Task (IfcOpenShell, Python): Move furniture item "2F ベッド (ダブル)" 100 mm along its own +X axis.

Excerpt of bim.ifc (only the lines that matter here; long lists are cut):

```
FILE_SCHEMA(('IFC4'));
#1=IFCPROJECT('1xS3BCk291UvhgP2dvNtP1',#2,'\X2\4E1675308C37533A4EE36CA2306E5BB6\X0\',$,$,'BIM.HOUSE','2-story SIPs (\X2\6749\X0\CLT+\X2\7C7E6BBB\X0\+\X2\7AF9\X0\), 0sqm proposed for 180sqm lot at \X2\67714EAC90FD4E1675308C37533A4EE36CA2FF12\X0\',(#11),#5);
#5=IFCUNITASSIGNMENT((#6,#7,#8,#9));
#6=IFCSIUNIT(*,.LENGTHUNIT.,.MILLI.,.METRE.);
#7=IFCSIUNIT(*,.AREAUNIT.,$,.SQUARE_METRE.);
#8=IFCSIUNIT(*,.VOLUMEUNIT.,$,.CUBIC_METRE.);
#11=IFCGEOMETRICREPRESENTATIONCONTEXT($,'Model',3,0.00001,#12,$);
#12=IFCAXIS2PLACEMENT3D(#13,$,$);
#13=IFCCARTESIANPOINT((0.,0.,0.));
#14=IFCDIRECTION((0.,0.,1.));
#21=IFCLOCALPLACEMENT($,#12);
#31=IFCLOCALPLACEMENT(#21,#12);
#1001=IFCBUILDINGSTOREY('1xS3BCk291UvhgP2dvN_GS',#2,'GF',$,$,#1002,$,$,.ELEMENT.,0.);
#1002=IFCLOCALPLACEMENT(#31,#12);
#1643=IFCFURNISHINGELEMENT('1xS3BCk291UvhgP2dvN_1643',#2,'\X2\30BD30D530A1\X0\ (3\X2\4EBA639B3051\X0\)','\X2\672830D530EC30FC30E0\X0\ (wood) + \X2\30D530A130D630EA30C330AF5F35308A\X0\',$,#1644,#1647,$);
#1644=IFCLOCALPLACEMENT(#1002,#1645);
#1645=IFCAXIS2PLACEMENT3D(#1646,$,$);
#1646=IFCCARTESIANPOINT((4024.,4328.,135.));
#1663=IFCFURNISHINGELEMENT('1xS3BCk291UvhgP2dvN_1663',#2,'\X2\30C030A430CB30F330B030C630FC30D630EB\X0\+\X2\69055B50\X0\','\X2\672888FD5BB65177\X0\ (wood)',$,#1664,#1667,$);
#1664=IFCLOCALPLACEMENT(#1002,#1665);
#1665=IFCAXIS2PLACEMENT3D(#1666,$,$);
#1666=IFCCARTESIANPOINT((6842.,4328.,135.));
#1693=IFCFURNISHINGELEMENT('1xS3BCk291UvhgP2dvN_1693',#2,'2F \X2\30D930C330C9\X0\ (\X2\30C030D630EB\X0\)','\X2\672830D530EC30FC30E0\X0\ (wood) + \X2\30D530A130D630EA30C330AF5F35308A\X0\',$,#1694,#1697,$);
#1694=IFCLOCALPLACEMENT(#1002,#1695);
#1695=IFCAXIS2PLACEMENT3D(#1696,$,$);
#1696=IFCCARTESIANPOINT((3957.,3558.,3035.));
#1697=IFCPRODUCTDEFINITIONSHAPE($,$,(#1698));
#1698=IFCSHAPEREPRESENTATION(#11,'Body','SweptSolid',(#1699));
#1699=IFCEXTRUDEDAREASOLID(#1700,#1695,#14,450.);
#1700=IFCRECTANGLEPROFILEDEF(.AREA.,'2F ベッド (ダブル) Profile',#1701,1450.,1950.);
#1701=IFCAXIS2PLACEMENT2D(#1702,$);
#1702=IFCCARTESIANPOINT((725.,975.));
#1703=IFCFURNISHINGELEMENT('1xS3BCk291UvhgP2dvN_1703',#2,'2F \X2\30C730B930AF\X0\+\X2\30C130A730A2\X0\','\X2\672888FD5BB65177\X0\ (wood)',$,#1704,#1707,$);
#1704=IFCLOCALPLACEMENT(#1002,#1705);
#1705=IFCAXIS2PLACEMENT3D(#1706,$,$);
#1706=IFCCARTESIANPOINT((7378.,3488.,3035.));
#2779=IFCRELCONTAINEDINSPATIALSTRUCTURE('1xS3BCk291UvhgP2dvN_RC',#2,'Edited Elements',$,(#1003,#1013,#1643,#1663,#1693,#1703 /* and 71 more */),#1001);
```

```python
import ifcopenshell
import ifcopenshell.api.geometry
import ifcopenshell.util.placement
import ifcopenshell.util.unit

model = ifcopenshell.open("bim.ifc")
unit_scale = ifcopenshell.util.unit.calculate_unit_scale(model)

item = model.by_id(1693)
matrix = ifcopenshell.util.placement.get_local_placement(item.ObjectPlacement)
matrix[:3, 3] += matrix[:3, 0] * 0.1 / unit_scale
ifcopenshell.api.geometry.edit_object_placement(model, product=item, matrix=matrix, is_si=False)

print(ifcopenshell.util.placement.get_local_placement(item.ObjectPlacement).round(3) + 0.0)

model.write("bim-out.ifc")
```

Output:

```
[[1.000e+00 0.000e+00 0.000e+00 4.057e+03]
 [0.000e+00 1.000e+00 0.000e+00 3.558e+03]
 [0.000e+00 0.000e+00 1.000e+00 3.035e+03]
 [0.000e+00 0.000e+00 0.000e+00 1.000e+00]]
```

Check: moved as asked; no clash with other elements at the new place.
